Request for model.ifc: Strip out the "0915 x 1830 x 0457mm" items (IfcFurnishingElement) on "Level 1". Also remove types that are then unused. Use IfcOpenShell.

First a look at what the model holds.

```python
import ifcopenshell
import ifcopenshell.util.element

model = ifcopenshell.open("model.ifc")
print(model.schema)
storey = next(s for s in model.by_type("IfcBuildingStorey") if s.Name == "Level 1")
furniture = [e for e in ifcopenshell.util.element.get_decomposition(storey) if e.is_a("IfcFurnishingElement")]
seen = {}
for e in furniture:
    element_type = ifcopenshell.util.element.get_type(e)
    name = element_type.Name if element_type not in (None, e) else None
    seen[name] = seen.get(name, 0) + 1
for name, count in sorted(seen.items(), key=str):
    print(count, "x", name)
```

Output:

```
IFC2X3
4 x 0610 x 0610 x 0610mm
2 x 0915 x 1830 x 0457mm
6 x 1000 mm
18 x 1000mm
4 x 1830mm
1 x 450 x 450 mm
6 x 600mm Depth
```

```python
import ifcopenshell
import ifcopenshell.api.root
import ifcopenshell.util.element

model = ifcopenshell.open("model.ifc")

storey = next(s for s in model.by_type("IfcBuildingStorey") if s.Name == "Level 1")
furniture = [e for e in ifcopenshell.util.element.get_decomposition(storey) if e.is_a("IfcFurnishingElement")]
targets = [e for e in furniture if (t := ifcopenshell.util.element.get_type(e)) not in (None, e) and t.Name == "0915 x 1830 x 0457mm"]
types = {ifcopenshell.util.element.get_type(e) for e in targets} - {None, *targets}

for e in targets:
    ifcopenshell.api.root.remove_product(model, product=e)
print(len(targets), "removed")

unused = [t for t in types if not ifcopenshell.util.element.get_types(t)]
for t in unused:
    ifcopenshell.api.root.remove_product(model, product=t)
print(len(unused), "unused types removed")

model.write("model_v2.ifc")
```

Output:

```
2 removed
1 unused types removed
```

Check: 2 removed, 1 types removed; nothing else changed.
